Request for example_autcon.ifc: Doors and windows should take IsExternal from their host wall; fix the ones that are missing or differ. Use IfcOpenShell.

First a look at what the model holds.

```python
import ifcopenshell
import ifcopenshell.util.element

model = ifcopenshell.open("example_autcon.ifc")
print(model.schema)
seen = {}
for e in model.by_type("IfcDoor") + model.by_type("IfcWindow"):
    if not e.FillsVoids:
        continue
    host = e.FillsVoids[0].RelatingOpeningElement.VoidsElements[0].RelatingBuildingElement
    own = ifcopenshell.util.element.get_pset(e, f"Pset_{e.is_a()[3:].removesuffix('StandardCase')}Common", "IsExternal")
    wall = ifcopenshell.util.element.get_pset(host, "Pset_WallCommon", "IsExternal")
    seen[e.is_a(), own, wall] = seen.get((e.is_a(), own, wall), 0) + 1
for (cls, own, wall), count in sorted(seen.items(), key=str):
    print(count, cls, "IsExternal:", own, "| host wall:", wall)
```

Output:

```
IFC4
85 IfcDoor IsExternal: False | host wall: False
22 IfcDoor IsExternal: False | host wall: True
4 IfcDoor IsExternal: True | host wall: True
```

```python
import ifcopenshell
import ifcopenshell.api.pset
import ifcopenshell.util.element

model = ifcopenshell.open("example_autcon.ifc")

count = 0
for ifc_class, pset_name in (("IfcDoor", "Pset_DoorCommon"), ("IfcWindow", "Pset_WindowCommon")):
    for e in model.by_type(ifc_class):
        if not e.FillsVoids:
            continue
        host = e.FillsVoids[0].RelatingOpeningElement.VoidsElements[0].RelatingBuildingElement
        external = ifcopenshell.util.element.get_pset(host, "Pset_WallCommon", "IsExternal")
        if external is None or ifcopenshell.util.element.get_pset(e, pset_name, "IsExternal") == external:
            continue
        pset = ifcopenshell.api.pset.add_pset(model, product=e, name=pset_name)
        ifcopenshell.api.pset.edit_pset(model, pset=pset, properties={"IsExternal": external})
        count += 1

print(count, "updated")

model.write("example_autcon_updated.ifc")
```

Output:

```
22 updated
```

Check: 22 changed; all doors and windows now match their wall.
